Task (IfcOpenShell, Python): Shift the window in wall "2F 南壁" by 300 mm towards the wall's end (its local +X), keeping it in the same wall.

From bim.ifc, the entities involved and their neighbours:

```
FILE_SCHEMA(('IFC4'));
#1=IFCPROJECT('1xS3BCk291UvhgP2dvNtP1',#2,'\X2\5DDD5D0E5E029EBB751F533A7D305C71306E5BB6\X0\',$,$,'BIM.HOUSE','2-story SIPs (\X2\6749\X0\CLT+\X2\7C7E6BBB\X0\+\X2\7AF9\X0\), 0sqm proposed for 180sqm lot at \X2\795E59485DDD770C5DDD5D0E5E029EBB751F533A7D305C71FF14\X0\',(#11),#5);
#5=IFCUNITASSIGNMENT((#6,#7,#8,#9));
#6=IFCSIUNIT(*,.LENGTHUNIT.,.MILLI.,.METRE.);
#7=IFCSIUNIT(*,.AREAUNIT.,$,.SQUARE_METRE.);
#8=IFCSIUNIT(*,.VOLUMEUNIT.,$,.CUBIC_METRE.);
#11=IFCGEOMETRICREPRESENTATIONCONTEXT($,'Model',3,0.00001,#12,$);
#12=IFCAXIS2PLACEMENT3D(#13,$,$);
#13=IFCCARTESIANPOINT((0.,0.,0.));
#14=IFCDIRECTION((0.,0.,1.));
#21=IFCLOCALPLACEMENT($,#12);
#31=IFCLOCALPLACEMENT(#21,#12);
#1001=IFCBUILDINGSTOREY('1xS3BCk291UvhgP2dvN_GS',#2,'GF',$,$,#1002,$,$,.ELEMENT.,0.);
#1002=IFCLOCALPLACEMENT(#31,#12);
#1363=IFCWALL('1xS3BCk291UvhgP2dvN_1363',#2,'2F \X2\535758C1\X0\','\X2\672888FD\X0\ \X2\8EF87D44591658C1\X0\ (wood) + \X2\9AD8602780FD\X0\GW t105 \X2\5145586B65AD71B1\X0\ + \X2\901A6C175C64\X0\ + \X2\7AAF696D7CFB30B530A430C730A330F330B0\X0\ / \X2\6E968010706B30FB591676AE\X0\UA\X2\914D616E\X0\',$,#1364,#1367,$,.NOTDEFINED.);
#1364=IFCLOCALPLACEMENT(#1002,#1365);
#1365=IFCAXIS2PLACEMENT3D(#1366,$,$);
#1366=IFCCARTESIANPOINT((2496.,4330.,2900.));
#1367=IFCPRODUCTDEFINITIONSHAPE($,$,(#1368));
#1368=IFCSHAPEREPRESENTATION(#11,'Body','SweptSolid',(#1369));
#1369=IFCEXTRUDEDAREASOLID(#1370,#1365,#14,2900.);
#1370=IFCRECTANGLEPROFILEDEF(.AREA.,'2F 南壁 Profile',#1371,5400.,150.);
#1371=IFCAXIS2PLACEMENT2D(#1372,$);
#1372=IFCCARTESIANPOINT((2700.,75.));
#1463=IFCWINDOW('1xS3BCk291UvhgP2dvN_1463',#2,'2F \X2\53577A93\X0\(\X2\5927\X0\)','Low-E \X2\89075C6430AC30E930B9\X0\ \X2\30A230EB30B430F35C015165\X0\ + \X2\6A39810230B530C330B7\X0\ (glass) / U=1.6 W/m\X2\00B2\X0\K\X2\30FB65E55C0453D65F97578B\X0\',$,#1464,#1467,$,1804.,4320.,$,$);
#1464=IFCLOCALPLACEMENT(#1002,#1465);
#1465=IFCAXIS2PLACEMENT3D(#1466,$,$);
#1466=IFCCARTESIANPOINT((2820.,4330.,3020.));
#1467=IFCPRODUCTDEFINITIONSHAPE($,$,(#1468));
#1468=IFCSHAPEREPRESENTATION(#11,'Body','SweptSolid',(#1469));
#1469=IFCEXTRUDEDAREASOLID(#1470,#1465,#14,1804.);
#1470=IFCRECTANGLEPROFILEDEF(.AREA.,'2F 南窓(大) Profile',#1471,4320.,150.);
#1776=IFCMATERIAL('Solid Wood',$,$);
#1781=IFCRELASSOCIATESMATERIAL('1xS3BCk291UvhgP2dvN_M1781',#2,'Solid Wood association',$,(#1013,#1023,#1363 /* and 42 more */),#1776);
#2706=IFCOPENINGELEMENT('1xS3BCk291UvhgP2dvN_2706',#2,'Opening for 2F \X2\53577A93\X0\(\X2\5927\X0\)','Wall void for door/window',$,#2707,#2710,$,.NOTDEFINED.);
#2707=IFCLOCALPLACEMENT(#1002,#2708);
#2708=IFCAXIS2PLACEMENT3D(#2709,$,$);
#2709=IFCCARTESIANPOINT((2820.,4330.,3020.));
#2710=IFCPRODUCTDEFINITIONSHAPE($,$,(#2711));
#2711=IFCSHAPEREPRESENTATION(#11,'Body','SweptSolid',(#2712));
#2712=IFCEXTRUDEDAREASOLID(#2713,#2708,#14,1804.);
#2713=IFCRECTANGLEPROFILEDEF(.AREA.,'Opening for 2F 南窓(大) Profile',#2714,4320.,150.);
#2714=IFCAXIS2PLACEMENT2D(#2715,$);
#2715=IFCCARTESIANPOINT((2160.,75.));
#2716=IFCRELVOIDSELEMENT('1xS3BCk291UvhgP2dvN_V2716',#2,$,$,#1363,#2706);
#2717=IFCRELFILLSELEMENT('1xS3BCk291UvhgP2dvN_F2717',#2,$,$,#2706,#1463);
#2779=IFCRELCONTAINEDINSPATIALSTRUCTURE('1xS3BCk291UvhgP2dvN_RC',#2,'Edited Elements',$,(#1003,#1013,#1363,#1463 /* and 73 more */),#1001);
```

```python
import ifcopenshell
import ifcopenshell.api.geometry
import ifcopenshell.util.placement
import ifcopenshell.util.unit

model = ifcopenshell.open("bim.ifc")
unit_scale = ifcopenshell.util.unit.calculate_unit_scale(model)

window = model.by_id(1463)
opening = window.FillsVoids[0].RelatingOpeningElement
wall = opening.VoidsElements[0].RelatingBuildingElement

wall_matrix = ifcopenshell.util.placement.get_local_placement(wall.ObjectPlacement)
shift = wall_matrix[:3, 0] * 0.3 / unit_scale
before = ifcopenshell.util.placement.get_local_placement(window.ObjectPlacement)[:3, 3].copy()

# The window is not placed relative to its opening, so move both.
for product in (opening, window):
    matrix = ifcopenshell.util.placement.get_local_placement(product.ObjectPlacement)
    matrix[:3, 3] += shift
    ifcopenshell.api.geometry.edit_object_placement(model, product=product, matrix=matrix, is_si=False)

after = ifcopenshell.util.placement.get_local_placement(window.ObjectPlacement)[:3, 3]
print("window moved by", (after - before).round(3) + 0.0)

model.write("bim-out.ifc")
```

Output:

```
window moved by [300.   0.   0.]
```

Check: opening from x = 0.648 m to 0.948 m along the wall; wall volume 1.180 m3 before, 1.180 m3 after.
